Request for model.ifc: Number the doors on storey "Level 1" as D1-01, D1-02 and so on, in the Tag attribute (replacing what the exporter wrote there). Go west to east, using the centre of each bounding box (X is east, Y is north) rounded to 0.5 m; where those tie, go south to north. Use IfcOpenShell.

First a look at what the model holds.

```python
import ifcopenshell
import ifcopenshell.util.element
import ifcopenshell.util.placement

model = ifcopenshell.open("model.ifc")
print(model.schema)
storey = next(s for s in model.by_type("IfcBuildingStorey") if s.Name == "Level 1")
doors = [e for e in ifcopenshell.util.element.get_decomposition(storey) if e.is_a("IfcDoor")]
for e in sorted(doors, key=lambda e: e.id()):
    origin = ifcopenshell.util.placement.get_local_placement(e.ObjectPlacement)[:3, 3]
    print(e.id(), e.Tag, e.Name, origin.round(2) + 0.0, sep=" | ")
```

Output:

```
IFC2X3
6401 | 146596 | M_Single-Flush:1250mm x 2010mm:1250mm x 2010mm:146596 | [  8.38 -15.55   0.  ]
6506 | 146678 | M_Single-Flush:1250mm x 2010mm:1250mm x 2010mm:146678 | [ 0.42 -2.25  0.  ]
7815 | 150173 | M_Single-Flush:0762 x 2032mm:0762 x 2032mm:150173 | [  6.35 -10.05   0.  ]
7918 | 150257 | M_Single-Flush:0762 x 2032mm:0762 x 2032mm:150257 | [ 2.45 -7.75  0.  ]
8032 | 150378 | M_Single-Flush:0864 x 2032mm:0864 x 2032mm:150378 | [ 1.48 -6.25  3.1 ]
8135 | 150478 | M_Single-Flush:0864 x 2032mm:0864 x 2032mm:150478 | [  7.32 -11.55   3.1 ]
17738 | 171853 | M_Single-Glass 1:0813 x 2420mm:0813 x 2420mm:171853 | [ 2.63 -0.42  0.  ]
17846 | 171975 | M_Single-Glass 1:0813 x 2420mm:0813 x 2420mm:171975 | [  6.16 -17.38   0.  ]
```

```python
import ifcopenshell
import ifcopenshell.geom
import ifcopenshell.util.element
import ifcopenshell.util.shape

model = ifcopenshell.open("model.ifc")
settings = ifcopenshell.geom.settings()
settings.set("use-world-coords", True)


def centre(element):
    shape = ifcopenshell.geom.create_shape(settings, element)
    return ifcopenshell.util.shape.get_bbox_centroid(shape.geometry)


storey = next(s for s in model.by_type("IfcBuildingStorey") if s.Name == "Level 1")
doors = [e for e in ifcopenshell.util.element.get_decomposition(storey) if e.is_a("IfcDoor")]

# Insertion points can sit at a corner or the storey origin, so sort by the geometry (in metres).
centres = {e: centre(e) for e in doors}
doors.sort(key=lambda e: (round(centres[e][0] / 0.5), centres[e][1]))

for i, e in enumerate(doors, start=1):
    number = f"D1-{i:02d}"
    e.Tag = number
    print(e.id(), number)

model.write("model_edited.ifc")
```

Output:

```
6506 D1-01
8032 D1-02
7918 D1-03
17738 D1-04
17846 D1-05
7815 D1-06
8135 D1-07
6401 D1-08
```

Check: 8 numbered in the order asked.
